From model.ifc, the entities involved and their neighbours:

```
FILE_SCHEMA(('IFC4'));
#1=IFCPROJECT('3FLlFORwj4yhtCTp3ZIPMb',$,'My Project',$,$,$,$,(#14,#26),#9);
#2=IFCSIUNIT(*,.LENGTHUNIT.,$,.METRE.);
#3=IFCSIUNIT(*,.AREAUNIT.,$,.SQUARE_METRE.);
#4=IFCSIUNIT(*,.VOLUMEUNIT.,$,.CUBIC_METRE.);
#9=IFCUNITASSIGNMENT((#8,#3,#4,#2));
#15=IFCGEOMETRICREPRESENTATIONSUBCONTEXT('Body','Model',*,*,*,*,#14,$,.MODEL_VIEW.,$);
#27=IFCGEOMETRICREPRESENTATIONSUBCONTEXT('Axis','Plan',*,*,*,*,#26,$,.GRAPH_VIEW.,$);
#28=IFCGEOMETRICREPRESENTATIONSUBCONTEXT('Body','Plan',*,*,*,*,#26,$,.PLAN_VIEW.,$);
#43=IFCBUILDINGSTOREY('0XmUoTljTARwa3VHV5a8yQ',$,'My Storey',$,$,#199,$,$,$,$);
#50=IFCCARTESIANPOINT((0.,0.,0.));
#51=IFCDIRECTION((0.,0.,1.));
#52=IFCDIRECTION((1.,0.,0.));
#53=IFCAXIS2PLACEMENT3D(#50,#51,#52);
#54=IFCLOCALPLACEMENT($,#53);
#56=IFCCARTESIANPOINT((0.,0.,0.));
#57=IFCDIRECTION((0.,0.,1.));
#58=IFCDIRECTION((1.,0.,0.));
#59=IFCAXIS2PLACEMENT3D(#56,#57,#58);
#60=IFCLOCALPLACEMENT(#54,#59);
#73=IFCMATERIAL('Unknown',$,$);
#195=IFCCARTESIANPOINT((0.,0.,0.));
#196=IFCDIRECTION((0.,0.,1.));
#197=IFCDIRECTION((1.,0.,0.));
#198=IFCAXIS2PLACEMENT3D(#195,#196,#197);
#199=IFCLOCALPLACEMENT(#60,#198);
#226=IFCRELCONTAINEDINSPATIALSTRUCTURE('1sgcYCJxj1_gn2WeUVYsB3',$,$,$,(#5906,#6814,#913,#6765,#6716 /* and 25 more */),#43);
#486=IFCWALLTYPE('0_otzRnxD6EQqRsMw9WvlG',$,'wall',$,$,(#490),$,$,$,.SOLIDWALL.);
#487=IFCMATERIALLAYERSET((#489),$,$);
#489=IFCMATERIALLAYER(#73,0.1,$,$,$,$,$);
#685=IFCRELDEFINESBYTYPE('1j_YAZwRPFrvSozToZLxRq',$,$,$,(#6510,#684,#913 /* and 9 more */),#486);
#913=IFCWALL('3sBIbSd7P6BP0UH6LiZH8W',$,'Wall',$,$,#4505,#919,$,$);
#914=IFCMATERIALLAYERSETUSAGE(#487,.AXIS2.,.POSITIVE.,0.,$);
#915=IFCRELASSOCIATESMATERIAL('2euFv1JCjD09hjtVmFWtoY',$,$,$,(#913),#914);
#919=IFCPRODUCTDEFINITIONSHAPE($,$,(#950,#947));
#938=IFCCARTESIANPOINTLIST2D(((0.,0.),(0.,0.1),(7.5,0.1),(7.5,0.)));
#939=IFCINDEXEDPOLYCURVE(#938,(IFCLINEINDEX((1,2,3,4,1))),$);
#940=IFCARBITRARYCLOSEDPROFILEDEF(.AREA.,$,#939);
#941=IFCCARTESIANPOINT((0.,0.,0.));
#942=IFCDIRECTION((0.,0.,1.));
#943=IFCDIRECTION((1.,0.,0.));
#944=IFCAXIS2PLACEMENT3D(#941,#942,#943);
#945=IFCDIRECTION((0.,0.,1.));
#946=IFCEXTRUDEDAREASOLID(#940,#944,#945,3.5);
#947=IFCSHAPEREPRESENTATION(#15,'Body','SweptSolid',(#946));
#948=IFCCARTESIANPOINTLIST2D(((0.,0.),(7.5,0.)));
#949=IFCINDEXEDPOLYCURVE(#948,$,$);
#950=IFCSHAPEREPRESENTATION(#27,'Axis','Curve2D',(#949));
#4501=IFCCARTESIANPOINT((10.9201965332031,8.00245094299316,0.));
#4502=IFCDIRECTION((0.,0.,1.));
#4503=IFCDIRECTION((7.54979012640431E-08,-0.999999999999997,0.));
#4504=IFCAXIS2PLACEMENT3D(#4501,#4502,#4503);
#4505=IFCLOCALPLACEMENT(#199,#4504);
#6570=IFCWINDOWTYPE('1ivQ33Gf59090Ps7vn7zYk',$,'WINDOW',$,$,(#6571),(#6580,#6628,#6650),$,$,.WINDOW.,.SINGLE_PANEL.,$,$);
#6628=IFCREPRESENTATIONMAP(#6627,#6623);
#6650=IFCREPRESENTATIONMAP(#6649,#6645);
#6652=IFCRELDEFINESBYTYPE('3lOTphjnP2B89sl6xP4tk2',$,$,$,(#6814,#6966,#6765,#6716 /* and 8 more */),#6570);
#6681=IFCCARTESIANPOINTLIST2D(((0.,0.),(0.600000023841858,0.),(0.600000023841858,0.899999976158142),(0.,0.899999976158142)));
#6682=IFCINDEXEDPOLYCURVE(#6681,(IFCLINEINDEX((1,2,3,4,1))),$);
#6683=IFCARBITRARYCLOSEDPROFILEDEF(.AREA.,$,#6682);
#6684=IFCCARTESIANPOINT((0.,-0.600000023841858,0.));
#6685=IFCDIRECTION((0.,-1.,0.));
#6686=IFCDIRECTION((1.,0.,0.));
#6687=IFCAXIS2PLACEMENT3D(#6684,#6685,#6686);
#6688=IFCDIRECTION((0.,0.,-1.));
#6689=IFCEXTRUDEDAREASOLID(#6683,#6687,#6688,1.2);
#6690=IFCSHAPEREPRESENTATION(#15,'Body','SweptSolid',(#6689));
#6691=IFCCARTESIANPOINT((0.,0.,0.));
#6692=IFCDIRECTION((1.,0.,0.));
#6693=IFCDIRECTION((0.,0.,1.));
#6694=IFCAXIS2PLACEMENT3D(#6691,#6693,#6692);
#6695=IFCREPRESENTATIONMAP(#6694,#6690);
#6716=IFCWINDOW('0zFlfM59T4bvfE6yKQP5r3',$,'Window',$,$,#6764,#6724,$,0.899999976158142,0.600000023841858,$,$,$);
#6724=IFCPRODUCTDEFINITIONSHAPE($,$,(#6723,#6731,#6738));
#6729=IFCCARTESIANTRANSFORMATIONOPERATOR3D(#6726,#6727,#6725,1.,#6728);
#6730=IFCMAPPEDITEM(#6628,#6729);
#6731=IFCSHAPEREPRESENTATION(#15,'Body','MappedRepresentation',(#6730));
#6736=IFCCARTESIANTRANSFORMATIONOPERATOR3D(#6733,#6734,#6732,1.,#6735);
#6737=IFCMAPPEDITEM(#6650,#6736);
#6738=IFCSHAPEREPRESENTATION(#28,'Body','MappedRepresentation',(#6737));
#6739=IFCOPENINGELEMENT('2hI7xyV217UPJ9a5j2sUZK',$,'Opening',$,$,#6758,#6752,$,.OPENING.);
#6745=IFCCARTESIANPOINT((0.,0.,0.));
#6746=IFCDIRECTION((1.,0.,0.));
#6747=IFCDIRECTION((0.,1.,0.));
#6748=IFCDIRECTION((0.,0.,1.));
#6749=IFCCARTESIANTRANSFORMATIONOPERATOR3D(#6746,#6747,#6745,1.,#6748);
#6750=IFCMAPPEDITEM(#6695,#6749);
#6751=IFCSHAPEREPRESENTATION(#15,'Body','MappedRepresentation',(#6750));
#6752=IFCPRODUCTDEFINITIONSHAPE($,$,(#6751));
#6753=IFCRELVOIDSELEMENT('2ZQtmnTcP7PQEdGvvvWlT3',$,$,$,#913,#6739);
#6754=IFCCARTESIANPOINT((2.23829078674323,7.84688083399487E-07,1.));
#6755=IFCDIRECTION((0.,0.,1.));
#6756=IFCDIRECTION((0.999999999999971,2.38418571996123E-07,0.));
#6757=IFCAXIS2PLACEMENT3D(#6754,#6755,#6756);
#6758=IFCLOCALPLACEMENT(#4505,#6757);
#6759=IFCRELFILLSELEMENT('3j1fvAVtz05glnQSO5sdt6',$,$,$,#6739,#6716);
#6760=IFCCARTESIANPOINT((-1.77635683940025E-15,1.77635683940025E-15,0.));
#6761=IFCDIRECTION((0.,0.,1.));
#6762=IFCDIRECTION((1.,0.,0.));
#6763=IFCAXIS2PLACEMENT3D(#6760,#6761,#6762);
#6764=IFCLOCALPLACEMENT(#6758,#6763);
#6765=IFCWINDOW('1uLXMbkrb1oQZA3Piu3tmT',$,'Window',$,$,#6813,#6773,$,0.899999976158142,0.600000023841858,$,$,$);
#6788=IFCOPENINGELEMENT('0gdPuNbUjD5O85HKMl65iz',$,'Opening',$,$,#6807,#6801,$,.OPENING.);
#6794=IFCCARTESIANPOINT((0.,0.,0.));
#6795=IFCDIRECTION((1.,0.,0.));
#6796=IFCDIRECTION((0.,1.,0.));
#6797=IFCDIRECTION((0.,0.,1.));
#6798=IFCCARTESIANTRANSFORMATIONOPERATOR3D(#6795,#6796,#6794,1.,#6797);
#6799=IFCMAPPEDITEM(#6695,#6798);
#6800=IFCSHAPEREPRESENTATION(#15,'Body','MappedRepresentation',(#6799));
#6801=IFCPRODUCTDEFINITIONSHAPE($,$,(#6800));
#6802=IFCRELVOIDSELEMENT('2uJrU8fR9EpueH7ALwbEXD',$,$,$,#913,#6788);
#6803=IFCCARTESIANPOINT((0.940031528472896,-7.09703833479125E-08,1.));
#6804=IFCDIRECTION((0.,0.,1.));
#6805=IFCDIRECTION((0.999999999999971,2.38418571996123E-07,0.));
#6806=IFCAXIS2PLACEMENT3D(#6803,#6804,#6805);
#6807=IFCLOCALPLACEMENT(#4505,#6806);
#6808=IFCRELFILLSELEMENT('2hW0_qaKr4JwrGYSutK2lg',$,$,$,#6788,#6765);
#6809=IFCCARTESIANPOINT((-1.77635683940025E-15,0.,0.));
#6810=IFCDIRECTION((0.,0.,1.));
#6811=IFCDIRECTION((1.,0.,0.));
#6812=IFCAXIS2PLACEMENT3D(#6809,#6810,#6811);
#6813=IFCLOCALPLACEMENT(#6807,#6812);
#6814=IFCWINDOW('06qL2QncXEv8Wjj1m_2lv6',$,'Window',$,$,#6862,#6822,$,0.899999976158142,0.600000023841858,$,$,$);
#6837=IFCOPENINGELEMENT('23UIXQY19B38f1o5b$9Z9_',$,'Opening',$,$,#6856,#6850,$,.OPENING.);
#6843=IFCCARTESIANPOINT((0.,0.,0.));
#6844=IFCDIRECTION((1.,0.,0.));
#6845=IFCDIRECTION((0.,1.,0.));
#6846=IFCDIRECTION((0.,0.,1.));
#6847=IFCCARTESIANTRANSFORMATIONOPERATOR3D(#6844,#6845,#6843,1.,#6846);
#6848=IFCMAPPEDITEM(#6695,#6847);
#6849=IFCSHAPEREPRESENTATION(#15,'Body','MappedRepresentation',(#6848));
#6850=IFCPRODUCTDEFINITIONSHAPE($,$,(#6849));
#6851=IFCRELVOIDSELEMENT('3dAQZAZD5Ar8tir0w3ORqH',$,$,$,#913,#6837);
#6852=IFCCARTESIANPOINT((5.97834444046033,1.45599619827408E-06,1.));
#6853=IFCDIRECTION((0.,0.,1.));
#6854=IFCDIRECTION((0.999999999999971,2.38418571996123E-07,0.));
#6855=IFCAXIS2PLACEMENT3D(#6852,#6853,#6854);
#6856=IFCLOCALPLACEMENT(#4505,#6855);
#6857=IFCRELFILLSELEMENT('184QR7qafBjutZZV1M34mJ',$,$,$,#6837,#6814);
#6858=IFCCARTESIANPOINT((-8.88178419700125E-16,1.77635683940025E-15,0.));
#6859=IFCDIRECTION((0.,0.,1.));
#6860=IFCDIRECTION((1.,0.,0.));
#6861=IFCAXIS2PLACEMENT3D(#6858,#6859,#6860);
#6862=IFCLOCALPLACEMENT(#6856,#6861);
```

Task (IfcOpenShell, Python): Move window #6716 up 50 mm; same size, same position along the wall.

```python
import numpy as np
import ifcopenshell
import ifcopenshell.api.geometry
import ifcopenshell.util.placement
import ifcopenshell.util.unit

model = ifcopenshell.open("model.ifc")
unit_scale = ifcopenshell.util.unit.calculate_unit_scale(model)

window = model.by_guid("0zFlfM59T4bvfE6yKQP5r3")
opening = window.FillsVoids[0].RelatingOpeningElement
dz = 0.05 / unit_scale

shift = np.array([0.0, 0.0, dz])
# The window is placed relative to its opening, so it follows when the opening moves.
matrix = ifcopenshell.util.placement.get_local_placement(opening.ObjectPlacement)
matrix[:3, 3] += shift
ifcopenshell.api.geometry.edit_object_placement(
    model, product=opening, matrix=matrix, is_si=False, should_transform_children=True
)

print(f"moved by {dz * unit_scale:+.3f} m")

model.write("model-out.ifc")
```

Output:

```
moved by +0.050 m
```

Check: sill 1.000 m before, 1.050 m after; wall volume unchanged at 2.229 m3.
